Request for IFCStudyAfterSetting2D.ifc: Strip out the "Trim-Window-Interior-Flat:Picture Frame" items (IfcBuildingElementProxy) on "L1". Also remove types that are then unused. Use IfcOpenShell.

First a look at what the model holds.

```python
import ifcopenshell
import ifcopenshell.util.element

model = ifcopenshell.open("IFCStudyAfterSetting2D.ifc")
print(model.schema)
storey = next(s for s in model.by_type("IfcBuildingStorey") if s.Name == "L1")
proxies = [e for e in ifcopenshell.util.element.get_decomposition(storey) if e.is_a("IfcBuildingElementProxy")]
seen = {}
for e in proxies:
    element_type = ifcopenshell.util.element.get_type(e)
    name = element_type.Name if element_type not in (None, e) else None
    seen[name] = seen.get(name, 0) + 1
for name, count in sorted(seen.items(), key=str):
    print(count, "x", name)
```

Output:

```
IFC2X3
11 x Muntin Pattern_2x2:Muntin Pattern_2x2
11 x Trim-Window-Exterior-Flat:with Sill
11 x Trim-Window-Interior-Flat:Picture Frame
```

```python
import ifcopenshell
import ifcopenshell.api.root
import ifcopenshell.util.element

model = ifcopenshell.open("IFCStudyAfterSetting2D.ifc")

storey = next(s for s in model.by_type("IfcBuildingStorey") if s.Name == "L1")
proxies = [e for e in ifcopenshell.util.element.get_decomposition(storey) if e.is_a("IfcBuildingElementProxy")]
targets = [e for e in proxies if (t := ifcopenshell.util.element.get_type(e)) not in (None, e) and t.Name == "Trim-Window-Interior-Flat:Picture Frame"]
types = {ifcopenshell.util.element.get_type(e) for e in targets} - {None, *targets}

for e in targets:
    ifcopenshell.api.root.remove_product(model, product=e)
print(len(targets), "removed")

unused = [t for t in types if not ifcopenshell.util.element.get_types(t)]
for t in unused:
    ifcopenshell.api.root.remove_product(model, product=t)
print(len(unused), "unused types removed")

model.write("IFCStudyAfterSetting2D_updated.ifc")
```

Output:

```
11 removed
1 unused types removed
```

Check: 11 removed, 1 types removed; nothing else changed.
